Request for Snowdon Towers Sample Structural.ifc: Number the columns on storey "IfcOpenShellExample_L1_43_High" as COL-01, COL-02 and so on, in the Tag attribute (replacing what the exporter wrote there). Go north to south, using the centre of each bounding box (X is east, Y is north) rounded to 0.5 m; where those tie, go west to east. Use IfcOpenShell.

First a look at what the model holds.

```python
import ifcopenshell
import ifcopenshell.util.element
import ifcopenshell.util.placement

model = ifcopenshell.open("Snowdon Towers Sample Structural.ifc")
print(model.schema)
storey = next(s for s in model.by_type("IfcBuildingStorey") if s.Name == "IfcOpenShellExample_L1_43_High")
columns = [e for e in ifcopenshell.util.element.get_decomposition(storey) if e.is_a("IfcColumn")]
for e in sorted(columns, key=lambda e: e.id()):
    origin = ifcopenshell.util.placement.get_local_placement(e.ObjectPlacement)[:3, 3]
    print(e.id(), e.Tag, e.Name, origin.round(2) + 0.0, sep=" | ")
```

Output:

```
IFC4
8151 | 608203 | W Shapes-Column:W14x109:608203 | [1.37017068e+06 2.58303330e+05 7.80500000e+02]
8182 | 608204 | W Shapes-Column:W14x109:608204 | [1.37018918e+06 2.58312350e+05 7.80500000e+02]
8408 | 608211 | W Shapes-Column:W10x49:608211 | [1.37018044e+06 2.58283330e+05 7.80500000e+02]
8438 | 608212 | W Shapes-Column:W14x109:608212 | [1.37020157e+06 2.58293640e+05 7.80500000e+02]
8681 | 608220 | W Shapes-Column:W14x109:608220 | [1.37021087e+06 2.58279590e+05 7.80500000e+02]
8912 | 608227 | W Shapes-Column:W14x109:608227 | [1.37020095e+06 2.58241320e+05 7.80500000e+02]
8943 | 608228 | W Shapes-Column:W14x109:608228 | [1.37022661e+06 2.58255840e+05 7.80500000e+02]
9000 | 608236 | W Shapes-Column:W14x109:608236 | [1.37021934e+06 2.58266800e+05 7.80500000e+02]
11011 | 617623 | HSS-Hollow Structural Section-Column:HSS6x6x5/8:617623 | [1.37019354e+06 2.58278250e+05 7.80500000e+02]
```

```python
import ifcopenshell
import ifcopenshell.geom
import ifcopenshell.util.element
import ifcopenshell.util.shape

model = ifcopenshell.open("Snowdon Towers Sample Structural.ifc")
settings = ifcopenshell.geom.settings()
settings.set("use-world-coords", True)


def centre(element):
    shape = ifcopenshell.geom.create_shape(settings, element)
    return ifcopenshell.util.shape.get_bbox_centroid(shape.geometry)


storey = next(s for s in model.by_type("IfcBuildingStorey") if s.Name == "IfcOpenShellExample_L1_43_High")
columns = [e for e in ifcopenshell.util.element.get_decomposition(storey) if e.is_a("IfcColumn")]

# Insertion points can sit at a corner or the storey origin, so sort by the geometry (in metres).
centres = {e: centre(e) for e in columns}
columns.sort(key=lambda e: (-round(centres[e][1] / 0.5), centres[e][0]))

for i, e in enumerate(columns, start=1):
    number = f"COL-{i:02d}"
    e.Tag = number
    print(e.id(), number)

model.write("Snowdon Towers Sample Structural_edited.ifc")
```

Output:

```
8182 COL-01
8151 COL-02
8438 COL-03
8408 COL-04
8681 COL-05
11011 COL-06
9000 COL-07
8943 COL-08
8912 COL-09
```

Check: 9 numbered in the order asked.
